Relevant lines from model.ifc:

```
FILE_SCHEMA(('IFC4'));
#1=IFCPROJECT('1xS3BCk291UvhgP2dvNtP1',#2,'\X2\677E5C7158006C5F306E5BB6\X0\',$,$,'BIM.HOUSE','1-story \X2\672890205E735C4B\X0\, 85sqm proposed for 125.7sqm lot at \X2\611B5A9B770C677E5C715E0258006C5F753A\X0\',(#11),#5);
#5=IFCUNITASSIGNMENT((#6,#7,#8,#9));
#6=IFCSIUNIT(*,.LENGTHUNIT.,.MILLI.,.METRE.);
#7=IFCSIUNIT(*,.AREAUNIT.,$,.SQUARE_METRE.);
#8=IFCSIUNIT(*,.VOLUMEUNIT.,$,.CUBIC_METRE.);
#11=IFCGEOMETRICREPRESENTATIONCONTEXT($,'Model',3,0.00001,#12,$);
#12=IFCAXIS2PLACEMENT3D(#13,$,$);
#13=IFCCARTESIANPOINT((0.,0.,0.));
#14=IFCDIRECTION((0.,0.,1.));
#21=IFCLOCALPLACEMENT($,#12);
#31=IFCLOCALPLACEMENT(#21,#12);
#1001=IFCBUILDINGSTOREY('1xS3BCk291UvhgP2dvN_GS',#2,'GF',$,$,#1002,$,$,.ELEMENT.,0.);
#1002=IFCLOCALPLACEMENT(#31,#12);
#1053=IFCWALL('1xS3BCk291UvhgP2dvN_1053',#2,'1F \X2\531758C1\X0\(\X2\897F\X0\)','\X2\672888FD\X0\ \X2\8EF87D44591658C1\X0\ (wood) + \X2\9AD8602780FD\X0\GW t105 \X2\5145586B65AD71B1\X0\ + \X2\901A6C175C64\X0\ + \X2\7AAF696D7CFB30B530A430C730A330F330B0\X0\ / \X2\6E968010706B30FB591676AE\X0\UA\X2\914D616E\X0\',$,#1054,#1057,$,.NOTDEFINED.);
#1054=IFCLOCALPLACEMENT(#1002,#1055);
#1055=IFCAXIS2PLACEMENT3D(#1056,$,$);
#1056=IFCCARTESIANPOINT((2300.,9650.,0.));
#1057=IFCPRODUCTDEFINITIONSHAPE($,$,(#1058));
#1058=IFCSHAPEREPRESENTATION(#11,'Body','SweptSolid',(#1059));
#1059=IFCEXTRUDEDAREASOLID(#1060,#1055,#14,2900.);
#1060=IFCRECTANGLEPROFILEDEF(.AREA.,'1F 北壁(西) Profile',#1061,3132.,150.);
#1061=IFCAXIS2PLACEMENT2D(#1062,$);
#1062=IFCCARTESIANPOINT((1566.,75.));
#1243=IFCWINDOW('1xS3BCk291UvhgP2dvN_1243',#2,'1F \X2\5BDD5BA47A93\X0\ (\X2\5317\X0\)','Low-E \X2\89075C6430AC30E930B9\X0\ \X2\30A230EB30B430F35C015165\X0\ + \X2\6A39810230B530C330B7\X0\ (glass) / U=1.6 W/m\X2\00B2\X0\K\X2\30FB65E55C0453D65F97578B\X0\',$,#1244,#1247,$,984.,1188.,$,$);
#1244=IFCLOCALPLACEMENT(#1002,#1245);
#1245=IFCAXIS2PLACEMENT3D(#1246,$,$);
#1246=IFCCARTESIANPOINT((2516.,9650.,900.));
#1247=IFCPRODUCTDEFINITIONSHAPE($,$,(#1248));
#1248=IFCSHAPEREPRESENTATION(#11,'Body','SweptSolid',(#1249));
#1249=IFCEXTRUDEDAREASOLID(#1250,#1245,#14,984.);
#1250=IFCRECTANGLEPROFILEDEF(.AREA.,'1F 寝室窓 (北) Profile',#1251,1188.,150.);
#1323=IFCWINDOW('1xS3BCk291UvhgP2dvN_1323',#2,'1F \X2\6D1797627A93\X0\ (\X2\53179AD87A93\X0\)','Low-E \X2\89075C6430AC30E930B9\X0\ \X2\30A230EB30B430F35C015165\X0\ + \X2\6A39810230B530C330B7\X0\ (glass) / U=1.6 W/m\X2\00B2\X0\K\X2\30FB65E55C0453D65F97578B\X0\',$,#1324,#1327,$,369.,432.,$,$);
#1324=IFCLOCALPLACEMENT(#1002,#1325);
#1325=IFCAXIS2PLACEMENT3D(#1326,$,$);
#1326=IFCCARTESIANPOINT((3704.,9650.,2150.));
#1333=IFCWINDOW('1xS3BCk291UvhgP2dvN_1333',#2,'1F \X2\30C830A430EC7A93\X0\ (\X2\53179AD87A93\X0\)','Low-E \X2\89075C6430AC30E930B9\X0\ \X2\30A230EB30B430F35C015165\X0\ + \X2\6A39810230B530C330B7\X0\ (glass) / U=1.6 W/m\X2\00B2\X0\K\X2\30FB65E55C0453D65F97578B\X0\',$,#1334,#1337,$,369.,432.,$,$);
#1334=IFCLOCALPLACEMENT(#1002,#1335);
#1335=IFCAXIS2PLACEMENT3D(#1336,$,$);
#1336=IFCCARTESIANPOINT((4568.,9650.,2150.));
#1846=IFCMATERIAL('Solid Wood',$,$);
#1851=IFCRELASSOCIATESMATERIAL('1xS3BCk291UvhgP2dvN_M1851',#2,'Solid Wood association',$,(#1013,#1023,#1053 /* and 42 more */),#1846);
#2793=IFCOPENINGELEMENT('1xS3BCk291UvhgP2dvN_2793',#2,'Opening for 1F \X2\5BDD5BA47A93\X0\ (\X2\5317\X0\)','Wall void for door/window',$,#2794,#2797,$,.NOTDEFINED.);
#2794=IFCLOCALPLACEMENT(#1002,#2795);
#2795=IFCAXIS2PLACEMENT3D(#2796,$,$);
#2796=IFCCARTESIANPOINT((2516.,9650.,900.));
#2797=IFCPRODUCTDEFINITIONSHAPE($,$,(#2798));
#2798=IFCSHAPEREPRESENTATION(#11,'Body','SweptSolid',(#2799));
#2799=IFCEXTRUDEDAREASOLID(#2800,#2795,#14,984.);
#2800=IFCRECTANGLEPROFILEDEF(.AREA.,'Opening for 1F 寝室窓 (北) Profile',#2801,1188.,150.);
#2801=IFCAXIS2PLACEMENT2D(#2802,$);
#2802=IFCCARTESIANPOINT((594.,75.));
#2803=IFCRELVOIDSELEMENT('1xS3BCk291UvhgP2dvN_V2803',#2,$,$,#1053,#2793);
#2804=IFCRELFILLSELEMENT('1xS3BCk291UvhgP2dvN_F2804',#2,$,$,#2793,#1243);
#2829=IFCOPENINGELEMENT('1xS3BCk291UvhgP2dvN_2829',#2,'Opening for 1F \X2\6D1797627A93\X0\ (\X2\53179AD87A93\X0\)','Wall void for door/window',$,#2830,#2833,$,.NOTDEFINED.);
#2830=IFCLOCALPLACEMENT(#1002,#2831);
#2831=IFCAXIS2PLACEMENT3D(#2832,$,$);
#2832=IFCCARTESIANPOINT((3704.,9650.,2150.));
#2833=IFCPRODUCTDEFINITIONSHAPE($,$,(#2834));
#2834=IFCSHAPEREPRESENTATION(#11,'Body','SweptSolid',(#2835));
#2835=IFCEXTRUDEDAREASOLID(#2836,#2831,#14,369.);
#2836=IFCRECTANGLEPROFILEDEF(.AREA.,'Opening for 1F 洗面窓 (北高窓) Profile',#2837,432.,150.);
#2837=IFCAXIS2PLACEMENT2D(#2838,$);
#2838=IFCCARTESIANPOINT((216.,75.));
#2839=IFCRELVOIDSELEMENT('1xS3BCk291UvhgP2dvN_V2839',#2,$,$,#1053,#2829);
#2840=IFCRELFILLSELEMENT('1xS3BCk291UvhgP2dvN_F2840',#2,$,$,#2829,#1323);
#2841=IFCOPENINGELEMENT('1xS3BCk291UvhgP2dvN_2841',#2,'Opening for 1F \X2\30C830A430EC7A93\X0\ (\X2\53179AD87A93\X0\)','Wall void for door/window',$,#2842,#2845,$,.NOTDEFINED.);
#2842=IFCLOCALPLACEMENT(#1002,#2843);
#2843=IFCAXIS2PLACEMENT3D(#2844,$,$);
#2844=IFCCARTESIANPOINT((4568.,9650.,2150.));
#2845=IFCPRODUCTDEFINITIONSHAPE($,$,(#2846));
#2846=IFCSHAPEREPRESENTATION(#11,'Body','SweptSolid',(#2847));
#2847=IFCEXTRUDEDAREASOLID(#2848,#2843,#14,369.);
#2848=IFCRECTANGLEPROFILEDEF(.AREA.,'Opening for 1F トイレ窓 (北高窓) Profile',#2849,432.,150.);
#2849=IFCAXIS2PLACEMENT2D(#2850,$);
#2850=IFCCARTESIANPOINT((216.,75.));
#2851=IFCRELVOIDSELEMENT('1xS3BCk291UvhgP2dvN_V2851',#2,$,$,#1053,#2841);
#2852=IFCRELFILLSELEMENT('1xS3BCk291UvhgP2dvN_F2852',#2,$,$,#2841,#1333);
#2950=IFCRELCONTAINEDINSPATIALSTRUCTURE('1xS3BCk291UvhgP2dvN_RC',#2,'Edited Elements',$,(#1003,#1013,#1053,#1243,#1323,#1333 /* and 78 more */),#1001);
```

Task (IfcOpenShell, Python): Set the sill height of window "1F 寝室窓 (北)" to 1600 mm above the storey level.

```python
import numpy as np
import ifcopenshell
import ifcopenshell.api.geometry
import ifcopenshell.geom
import ifcopenshell.util.element
import ifcopenshell.util.placement
import ifcopenshell.util.shape
import ifcopenshell.util.unit

model = ifcopenshell.open("model.ifc")
unit_scale = ifcopenshell.util.unit.calculate_unit_scale(model)

window = model.by_guid("1xS3BCk291UvhgP2dvN_1243")
opening = window.FillsVoids[0].RelatingOpeningElement
storey = ifcopenshell.util.element.get_container(window, ifc_class="IfcBuildingStorey")
level = ifcopenshell.util.placement.get_local_placement(storey.ObjectPlacement)[2, 3]

# The opening's origin need not be at the sill, so measure its lowest point.
shape = ifcopenshell.geom.create_shape(ifcopenshell.geom.settings(), opening)
bottom = ifcopenshell.util.shape.get_shape_bottom_elevation(shape, shape.geometry) / unit_scale
dz = level + 1.6 / unit_scale - bottom

shift = np.array([0.0, 0.0, dz])
# The window is not placed relative to its opening, so move both.
for product in (opening, window):
    matrix = ifcopenshell.util.placement.get_local_placement(product.ObjectPlacement)
    matrix[:3, 3] += shift
    ifcopenshell.api.geometry.edit_object_placement(model, product=product, matrix=matrix, is_si=False)

print(f"moved by {dz * unit_scale:+.3f} m")

model.write("model_edited.ifc")
```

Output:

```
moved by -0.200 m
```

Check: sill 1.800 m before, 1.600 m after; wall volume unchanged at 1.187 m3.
